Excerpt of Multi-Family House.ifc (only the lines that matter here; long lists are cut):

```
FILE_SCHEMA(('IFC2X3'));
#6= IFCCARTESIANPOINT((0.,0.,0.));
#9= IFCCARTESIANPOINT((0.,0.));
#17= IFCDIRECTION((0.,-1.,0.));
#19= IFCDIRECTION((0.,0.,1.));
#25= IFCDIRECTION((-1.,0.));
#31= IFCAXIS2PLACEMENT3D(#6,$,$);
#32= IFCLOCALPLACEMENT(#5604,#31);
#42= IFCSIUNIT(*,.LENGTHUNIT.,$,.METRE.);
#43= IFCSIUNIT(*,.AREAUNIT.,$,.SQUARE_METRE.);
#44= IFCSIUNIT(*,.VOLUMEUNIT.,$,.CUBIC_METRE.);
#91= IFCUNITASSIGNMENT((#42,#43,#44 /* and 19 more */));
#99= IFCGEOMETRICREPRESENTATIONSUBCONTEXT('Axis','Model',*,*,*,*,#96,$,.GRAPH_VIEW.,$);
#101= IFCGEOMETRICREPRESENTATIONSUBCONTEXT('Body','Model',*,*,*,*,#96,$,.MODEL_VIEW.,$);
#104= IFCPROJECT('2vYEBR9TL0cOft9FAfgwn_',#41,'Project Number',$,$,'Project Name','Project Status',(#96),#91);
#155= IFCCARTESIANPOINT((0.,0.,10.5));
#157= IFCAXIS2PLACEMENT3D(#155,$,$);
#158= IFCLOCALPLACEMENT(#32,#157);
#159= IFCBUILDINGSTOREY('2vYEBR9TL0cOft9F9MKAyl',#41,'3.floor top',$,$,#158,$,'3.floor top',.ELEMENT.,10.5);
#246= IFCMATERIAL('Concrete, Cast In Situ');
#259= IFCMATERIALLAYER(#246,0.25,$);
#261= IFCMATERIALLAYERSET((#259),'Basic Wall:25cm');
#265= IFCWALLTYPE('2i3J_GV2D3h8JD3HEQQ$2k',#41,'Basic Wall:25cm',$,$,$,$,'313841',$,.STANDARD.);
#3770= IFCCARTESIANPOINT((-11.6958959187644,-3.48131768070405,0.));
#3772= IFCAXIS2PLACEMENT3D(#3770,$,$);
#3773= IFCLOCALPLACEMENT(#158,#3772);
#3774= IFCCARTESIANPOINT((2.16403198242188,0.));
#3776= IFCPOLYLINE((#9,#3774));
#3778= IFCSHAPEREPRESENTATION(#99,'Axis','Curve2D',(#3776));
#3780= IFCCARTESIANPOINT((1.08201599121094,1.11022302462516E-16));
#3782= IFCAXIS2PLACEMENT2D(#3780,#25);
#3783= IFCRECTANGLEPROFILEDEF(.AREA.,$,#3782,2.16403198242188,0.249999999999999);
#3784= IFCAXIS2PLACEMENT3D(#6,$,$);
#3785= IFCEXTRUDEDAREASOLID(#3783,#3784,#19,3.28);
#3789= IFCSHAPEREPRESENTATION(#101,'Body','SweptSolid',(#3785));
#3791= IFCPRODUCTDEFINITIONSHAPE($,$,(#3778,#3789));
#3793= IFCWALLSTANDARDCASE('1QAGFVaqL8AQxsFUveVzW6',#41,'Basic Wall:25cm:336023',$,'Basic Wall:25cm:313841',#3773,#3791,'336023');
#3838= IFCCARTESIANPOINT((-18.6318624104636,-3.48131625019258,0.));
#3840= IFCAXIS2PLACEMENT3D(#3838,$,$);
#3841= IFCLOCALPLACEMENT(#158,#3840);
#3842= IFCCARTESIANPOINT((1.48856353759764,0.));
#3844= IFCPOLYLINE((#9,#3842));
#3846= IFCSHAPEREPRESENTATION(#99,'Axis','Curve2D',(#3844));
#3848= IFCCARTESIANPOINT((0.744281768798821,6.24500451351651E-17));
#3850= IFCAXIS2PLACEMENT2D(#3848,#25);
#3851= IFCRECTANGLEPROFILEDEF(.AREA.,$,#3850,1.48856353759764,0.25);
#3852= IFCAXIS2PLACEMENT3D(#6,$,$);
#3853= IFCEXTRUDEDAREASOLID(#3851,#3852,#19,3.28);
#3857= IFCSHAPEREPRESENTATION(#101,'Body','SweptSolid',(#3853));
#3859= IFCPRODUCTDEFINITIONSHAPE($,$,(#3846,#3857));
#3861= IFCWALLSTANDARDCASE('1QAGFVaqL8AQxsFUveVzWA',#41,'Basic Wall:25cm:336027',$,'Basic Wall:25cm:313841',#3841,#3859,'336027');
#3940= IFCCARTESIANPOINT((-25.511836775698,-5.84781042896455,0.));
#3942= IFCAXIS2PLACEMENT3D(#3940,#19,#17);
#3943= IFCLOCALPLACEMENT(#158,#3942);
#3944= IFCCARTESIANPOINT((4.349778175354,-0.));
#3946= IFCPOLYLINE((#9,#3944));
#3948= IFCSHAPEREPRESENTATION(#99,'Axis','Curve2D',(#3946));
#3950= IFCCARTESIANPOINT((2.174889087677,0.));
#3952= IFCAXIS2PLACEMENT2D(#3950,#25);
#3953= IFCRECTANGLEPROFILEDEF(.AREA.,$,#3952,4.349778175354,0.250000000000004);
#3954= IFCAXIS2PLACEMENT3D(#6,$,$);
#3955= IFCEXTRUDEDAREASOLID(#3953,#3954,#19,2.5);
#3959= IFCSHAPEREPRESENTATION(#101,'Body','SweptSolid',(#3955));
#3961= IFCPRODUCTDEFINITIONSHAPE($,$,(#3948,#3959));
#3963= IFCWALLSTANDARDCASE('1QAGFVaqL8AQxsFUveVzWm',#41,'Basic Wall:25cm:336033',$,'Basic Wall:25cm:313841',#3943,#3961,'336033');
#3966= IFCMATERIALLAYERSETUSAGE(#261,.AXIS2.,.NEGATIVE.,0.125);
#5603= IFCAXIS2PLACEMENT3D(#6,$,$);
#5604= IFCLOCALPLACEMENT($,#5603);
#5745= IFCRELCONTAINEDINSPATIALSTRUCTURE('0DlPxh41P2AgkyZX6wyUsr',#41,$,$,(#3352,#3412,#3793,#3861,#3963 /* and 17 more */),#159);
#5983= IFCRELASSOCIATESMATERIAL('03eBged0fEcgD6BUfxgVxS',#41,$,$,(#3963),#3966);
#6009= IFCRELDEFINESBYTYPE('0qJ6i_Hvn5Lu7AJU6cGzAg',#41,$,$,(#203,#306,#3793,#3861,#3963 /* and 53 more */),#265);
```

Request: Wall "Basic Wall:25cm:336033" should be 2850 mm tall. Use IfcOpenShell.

```python
import ifcopenshell
import ifcopenshell.geom
import ifcopenshell.util.representation
import ifcopenshell.util.shape
import ifcopenshell.util.unit

model = ifcopenshell.open("Multi-Family House.ifc")
unit_scale = ifcopenshell.util.unit.calculate_unit_scale(model)
settings = ifcopenshell.geom.settings()


def volume(element):
    """Net volume in cubic metres, openings subtracted."""
    shape = ifcopenshell.geom.create_shape(settings, element)
    return ifcopenshell.util.shape.get_volume(shape.geometry)


wall = model.by_id(3963)
before = volume(wall)

body = ifcopenshell.util.representation.get_representation(wall, "Model", "Body")
solid = body.Items[0]
old_height = solid.Depth
solid.Depth = 2.85 / unit_scale
after = volume(wall)

print(f"height {old_height:g} -> {solid.Depth:g}, volume {before:.3f} -> {after:.3f} m3")

model.write("Multi-Family House-out.ifc")
```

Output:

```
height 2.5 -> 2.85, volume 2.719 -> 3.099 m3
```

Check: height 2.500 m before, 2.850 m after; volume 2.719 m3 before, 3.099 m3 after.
